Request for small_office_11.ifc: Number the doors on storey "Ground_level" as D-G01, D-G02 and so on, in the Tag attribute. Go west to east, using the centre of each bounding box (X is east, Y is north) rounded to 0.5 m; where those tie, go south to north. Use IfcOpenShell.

First a look at what the model holds.

```python
import ifcopenshell
import ifcopenshell.util.element
import ifcopenshell.util.placement

model = ifcopenshell.open("small_office_11.ifc")
print(model.schema)
storey = next(s for s in model.by_type("IfcBuildingStorey") if s.Name == "Ground_level")
doors = [e for e in ifcopenshell.util.element.get_decomposition(storey) if e.is_a("IfcDoor")]
for e in sorted(doors, key=lambda e: e.id()):
    origin = ifcopenshell.util.placement.get_local_placement(e.ObjectPlacement)[:3, 3]
    print(e.id(), e.Tag, e.Name, origin.round(2) + 0.0, sep=" | ")
```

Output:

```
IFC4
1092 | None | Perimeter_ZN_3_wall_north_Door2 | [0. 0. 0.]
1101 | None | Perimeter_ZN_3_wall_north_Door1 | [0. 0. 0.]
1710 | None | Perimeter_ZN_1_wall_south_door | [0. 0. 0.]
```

```python
import ifcopenshell
import ifcopenshell.geom
import ifcopenshell.util.element
import ifcopenshell.util.shape

model = ifcopenshell.open("small_office_11.ifc")
settings = ifcopenshell.geom.settings()
settings.set("use-world-coords", True)


def centre(element):
    shape = ifcopenshell.geom.create_shape(settings, element)
    return ifcopenshell.util.shape.get_bbox_centroid(shape.geometry)


storey = next(s for s in model.by_type("IfcBuildingStorey") if s.Name == "Ground_level")
doors = [e for e in ifcopenshell.util.element.get_decomposition(storey) if e.is_a("IfcDoor")]

# Insertion points can sit at a corner or the storey origin, so sort by the geometry (in metres).
centres = {e: centre(e) for e in doors}
doors.sort(key=lambda e: (round(centres[e][0] / 0.5), centres[e][1]))

for i, e in enumerate(doors, start=1):
    number = f"D-G{i:02d}"
    e.Tag = number
    print(e.id(), number)

model.write("small_office_11-out.ifc")
```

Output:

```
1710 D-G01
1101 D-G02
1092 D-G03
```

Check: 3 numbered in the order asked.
